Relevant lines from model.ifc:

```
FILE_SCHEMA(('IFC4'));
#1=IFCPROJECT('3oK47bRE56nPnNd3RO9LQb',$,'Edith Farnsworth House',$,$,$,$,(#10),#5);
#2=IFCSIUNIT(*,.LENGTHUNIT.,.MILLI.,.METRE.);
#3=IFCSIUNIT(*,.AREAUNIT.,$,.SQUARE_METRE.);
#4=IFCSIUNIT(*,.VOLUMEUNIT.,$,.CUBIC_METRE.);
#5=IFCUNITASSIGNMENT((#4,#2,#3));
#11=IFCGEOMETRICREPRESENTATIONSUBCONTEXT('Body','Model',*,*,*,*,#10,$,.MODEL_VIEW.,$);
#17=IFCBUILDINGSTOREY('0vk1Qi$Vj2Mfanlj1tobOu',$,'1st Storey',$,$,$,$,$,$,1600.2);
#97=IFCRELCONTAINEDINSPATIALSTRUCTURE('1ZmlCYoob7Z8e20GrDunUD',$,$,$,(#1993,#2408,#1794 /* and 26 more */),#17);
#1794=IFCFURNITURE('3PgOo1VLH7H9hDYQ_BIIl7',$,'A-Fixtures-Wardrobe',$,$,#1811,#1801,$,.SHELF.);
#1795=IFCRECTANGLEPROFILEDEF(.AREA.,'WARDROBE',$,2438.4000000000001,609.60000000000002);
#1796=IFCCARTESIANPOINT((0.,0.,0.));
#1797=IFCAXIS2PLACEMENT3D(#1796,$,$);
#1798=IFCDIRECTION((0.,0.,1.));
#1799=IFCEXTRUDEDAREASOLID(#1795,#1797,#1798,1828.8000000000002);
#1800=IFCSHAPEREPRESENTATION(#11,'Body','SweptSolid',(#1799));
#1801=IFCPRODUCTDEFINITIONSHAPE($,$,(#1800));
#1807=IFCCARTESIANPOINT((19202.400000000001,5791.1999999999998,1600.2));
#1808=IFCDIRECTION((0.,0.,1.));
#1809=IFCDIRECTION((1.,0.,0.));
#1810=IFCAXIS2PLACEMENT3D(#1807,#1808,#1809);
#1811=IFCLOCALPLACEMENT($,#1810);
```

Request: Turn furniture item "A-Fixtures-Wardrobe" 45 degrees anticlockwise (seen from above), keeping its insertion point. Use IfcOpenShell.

```python
import ifcopenshell
import ifcopenshell.api.geometry
import ifcopenshell.util.placement

model = ifcopenshell.open("model.ifc")

item = model.by_guid("3PgOo1VLH7H9hDYQ_BIIl7")
matrix = ifcopenshell.util.placement.get_local_placement(item.ObjectPlacement)
matrix = matrix @ ifcopenshell.util.placement.rotation(45, "Z")
ifcopenshell.api.geometry.edit_object_placement(model, product=item, matrix=matrix, is_si=False)

print(ifcopenshell.util.placement.get_local_placement(item.ObjectPlacement).round(3) + 0.0)

model.write("model_v2.ifc")
```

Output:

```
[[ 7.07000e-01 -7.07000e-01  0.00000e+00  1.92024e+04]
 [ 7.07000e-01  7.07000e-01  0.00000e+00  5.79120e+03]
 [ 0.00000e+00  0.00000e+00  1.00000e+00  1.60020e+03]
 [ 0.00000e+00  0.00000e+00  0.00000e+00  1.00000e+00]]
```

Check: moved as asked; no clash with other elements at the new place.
